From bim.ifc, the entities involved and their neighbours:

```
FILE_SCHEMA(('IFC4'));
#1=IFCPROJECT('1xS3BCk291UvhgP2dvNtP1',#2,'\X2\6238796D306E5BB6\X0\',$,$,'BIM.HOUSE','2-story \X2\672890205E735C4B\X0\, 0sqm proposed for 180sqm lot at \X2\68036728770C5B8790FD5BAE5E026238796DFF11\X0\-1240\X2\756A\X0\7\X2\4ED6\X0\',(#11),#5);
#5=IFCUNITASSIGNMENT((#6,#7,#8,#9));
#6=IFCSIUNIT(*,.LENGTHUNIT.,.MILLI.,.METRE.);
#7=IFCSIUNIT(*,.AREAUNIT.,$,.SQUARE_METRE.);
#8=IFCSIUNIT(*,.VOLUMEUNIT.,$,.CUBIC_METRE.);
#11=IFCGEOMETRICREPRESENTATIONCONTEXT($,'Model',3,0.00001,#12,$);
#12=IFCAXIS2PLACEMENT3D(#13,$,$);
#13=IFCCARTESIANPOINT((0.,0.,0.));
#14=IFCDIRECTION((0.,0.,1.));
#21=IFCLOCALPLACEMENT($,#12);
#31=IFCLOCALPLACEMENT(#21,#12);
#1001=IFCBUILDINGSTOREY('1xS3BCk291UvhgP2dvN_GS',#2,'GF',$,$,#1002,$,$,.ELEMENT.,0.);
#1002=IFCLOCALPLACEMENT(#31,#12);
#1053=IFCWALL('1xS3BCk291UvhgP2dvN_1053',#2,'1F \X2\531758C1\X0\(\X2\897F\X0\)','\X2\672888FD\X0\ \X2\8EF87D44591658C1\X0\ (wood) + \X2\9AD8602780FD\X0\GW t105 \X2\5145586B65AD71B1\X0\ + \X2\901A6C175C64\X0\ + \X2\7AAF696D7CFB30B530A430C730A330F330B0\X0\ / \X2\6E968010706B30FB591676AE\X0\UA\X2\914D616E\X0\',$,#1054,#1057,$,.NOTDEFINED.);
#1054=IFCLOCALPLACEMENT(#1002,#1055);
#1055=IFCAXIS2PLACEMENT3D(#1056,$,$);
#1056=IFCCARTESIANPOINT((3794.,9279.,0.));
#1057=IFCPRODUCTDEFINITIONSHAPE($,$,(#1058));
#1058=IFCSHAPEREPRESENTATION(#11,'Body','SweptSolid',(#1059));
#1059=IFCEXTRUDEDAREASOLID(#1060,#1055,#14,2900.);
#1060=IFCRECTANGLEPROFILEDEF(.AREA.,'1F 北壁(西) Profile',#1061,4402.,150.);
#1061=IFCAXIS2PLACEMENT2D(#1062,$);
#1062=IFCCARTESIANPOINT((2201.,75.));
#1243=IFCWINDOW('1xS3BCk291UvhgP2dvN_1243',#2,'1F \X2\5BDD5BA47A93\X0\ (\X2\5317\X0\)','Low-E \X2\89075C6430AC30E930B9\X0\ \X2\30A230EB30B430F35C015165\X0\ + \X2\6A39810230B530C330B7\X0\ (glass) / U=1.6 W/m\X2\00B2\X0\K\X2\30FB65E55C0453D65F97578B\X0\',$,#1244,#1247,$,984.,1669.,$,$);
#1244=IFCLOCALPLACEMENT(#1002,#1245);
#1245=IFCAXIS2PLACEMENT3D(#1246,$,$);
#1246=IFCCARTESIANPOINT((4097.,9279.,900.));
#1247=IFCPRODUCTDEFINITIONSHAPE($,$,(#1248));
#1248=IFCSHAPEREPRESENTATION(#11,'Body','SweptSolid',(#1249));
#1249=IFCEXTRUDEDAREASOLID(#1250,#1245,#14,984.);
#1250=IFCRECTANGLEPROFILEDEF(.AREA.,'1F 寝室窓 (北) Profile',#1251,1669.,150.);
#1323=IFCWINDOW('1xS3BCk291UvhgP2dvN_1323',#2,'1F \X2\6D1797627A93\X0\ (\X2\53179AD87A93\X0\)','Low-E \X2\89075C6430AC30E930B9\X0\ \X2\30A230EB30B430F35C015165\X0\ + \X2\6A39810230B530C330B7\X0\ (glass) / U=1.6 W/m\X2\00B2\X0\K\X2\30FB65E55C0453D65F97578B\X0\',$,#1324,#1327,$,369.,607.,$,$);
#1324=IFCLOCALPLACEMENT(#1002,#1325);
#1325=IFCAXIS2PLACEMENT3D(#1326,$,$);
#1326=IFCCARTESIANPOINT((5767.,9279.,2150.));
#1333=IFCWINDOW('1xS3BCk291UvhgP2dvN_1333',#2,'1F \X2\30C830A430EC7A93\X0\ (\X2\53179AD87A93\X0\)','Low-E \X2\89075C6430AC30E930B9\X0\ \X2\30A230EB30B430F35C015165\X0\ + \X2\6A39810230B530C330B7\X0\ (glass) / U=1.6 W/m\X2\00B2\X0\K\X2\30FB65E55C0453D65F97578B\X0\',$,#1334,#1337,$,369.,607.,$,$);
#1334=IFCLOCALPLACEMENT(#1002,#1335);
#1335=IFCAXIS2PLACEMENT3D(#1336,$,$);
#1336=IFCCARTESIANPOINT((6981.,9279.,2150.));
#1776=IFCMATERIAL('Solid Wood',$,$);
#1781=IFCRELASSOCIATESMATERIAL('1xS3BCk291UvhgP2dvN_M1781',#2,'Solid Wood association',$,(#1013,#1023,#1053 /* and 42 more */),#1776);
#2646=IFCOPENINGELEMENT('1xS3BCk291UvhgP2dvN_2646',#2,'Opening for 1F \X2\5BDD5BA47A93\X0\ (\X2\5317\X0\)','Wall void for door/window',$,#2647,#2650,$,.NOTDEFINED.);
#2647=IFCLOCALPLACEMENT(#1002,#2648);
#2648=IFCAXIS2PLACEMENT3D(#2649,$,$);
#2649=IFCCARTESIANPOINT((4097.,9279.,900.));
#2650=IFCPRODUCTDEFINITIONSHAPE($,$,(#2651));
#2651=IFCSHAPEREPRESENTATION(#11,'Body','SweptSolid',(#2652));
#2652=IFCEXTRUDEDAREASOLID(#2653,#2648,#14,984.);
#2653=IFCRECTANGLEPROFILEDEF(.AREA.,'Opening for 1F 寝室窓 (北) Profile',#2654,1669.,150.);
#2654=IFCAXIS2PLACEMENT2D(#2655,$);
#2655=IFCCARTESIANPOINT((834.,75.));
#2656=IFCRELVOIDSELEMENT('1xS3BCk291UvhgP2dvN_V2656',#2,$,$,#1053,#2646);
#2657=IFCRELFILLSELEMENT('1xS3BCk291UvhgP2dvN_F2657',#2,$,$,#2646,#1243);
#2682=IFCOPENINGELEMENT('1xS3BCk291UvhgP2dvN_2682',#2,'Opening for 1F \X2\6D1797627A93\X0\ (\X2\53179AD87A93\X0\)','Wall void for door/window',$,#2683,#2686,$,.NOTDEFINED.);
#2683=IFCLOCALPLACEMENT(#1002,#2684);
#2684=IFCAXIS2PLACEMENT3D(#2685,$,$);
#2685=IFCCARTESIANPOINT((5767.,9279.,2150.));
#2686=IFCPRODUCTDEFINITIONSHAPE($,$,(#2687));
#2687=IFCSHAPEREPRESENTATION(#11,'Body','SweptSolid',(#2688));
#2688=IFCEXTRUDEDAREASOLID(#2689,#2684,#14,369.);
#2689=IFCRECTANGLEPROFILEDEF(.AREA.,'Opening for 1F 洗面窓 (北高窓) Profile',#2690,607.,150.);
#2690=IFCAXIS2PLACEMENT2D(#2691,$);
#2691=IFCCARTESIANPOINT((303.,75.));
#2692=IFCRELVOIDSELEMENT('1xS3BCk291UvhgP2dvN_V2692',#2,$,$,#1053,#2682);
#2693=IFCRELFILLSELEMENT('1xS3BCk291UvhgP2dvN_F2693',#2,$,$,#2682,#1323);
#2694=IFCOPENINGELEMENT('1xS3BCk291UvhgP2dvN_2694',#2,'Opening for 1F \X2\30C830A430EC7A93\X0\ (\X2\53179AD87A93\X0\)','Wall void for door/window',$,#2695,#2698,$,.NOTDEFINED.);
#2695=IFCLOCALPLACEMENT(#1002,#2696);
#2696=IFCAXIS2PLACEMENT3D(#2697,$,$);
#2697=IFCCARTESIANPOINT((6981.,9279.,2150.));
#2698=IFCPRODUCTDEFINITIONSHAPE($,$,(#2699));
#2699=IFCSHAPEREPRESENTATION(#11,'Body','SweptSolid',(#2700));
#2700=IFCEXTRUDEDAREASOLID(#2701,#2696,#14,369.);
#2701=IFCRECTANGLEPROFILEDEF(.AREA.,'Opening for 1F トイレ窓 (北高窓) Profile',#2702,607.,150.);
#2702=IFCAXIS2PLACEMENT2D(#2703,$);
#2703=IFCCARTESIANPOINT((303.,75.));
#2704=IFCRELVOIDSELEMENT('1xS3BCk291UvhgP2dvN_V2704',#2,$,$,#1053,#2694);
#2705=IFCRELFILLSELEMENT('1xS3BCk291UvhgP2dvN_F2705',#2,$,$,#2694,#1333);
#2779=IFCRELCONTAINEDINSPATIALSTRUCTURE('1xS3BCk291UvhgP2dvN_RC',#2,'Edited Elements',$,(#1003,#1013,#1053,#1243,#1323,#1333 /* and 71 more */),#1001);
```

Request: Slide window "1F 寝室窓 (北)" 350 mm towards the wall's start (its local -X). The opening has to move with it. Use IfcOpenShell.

```python
import ifcopenshell
import ifcopenshell.api.geometry
import ifcopenshell.util.placement
import ifcopenshell.util.unit

model = ifcopenshell.open("bim.ifc")
unit_scale = ifcopenshell.util.unit.calculate_unit_scale(model)

window = model.by_guid("1xS3BCk291UvhgP2dvN_1243")
opening = window.FillsVoids[0].RelatingOpeningElement
wall = opening.VoidsElements[0].RelatingBuildingElement

wall_matrix = ifcopenshell.util.placement.get_local_placement(wall.ObjectPlacement)
shift = wall_matrix[:3, 0] * -0.35 / unit_scale
before = ifcopenshell.util.placement.get_local_placement(window.ObjectPlacement)[:3, 3].copy()

# The window is not placed relative to its opening, so move both.
for product in (opening, window):
    matrix = ifcopenshell.util.placement.get_local_placement(product.ObjectPlacement)
    matrix[:3, 3] += shift
    ifcopenshell.api.geometry.edit_object_placement(model, product=product, matrix=matrix, is_si=False)

after = ifcopenshell.util.placement.get_local_placement(window.ObjectPlacement)[:3, 3]
print("window moved by", (after - before).round(3) + 0.0)

model.write("bim_edited.ifc")
```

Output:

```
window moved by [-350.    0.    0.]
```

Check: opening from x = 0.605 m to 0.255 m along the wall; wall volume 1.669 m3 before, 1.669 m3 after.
